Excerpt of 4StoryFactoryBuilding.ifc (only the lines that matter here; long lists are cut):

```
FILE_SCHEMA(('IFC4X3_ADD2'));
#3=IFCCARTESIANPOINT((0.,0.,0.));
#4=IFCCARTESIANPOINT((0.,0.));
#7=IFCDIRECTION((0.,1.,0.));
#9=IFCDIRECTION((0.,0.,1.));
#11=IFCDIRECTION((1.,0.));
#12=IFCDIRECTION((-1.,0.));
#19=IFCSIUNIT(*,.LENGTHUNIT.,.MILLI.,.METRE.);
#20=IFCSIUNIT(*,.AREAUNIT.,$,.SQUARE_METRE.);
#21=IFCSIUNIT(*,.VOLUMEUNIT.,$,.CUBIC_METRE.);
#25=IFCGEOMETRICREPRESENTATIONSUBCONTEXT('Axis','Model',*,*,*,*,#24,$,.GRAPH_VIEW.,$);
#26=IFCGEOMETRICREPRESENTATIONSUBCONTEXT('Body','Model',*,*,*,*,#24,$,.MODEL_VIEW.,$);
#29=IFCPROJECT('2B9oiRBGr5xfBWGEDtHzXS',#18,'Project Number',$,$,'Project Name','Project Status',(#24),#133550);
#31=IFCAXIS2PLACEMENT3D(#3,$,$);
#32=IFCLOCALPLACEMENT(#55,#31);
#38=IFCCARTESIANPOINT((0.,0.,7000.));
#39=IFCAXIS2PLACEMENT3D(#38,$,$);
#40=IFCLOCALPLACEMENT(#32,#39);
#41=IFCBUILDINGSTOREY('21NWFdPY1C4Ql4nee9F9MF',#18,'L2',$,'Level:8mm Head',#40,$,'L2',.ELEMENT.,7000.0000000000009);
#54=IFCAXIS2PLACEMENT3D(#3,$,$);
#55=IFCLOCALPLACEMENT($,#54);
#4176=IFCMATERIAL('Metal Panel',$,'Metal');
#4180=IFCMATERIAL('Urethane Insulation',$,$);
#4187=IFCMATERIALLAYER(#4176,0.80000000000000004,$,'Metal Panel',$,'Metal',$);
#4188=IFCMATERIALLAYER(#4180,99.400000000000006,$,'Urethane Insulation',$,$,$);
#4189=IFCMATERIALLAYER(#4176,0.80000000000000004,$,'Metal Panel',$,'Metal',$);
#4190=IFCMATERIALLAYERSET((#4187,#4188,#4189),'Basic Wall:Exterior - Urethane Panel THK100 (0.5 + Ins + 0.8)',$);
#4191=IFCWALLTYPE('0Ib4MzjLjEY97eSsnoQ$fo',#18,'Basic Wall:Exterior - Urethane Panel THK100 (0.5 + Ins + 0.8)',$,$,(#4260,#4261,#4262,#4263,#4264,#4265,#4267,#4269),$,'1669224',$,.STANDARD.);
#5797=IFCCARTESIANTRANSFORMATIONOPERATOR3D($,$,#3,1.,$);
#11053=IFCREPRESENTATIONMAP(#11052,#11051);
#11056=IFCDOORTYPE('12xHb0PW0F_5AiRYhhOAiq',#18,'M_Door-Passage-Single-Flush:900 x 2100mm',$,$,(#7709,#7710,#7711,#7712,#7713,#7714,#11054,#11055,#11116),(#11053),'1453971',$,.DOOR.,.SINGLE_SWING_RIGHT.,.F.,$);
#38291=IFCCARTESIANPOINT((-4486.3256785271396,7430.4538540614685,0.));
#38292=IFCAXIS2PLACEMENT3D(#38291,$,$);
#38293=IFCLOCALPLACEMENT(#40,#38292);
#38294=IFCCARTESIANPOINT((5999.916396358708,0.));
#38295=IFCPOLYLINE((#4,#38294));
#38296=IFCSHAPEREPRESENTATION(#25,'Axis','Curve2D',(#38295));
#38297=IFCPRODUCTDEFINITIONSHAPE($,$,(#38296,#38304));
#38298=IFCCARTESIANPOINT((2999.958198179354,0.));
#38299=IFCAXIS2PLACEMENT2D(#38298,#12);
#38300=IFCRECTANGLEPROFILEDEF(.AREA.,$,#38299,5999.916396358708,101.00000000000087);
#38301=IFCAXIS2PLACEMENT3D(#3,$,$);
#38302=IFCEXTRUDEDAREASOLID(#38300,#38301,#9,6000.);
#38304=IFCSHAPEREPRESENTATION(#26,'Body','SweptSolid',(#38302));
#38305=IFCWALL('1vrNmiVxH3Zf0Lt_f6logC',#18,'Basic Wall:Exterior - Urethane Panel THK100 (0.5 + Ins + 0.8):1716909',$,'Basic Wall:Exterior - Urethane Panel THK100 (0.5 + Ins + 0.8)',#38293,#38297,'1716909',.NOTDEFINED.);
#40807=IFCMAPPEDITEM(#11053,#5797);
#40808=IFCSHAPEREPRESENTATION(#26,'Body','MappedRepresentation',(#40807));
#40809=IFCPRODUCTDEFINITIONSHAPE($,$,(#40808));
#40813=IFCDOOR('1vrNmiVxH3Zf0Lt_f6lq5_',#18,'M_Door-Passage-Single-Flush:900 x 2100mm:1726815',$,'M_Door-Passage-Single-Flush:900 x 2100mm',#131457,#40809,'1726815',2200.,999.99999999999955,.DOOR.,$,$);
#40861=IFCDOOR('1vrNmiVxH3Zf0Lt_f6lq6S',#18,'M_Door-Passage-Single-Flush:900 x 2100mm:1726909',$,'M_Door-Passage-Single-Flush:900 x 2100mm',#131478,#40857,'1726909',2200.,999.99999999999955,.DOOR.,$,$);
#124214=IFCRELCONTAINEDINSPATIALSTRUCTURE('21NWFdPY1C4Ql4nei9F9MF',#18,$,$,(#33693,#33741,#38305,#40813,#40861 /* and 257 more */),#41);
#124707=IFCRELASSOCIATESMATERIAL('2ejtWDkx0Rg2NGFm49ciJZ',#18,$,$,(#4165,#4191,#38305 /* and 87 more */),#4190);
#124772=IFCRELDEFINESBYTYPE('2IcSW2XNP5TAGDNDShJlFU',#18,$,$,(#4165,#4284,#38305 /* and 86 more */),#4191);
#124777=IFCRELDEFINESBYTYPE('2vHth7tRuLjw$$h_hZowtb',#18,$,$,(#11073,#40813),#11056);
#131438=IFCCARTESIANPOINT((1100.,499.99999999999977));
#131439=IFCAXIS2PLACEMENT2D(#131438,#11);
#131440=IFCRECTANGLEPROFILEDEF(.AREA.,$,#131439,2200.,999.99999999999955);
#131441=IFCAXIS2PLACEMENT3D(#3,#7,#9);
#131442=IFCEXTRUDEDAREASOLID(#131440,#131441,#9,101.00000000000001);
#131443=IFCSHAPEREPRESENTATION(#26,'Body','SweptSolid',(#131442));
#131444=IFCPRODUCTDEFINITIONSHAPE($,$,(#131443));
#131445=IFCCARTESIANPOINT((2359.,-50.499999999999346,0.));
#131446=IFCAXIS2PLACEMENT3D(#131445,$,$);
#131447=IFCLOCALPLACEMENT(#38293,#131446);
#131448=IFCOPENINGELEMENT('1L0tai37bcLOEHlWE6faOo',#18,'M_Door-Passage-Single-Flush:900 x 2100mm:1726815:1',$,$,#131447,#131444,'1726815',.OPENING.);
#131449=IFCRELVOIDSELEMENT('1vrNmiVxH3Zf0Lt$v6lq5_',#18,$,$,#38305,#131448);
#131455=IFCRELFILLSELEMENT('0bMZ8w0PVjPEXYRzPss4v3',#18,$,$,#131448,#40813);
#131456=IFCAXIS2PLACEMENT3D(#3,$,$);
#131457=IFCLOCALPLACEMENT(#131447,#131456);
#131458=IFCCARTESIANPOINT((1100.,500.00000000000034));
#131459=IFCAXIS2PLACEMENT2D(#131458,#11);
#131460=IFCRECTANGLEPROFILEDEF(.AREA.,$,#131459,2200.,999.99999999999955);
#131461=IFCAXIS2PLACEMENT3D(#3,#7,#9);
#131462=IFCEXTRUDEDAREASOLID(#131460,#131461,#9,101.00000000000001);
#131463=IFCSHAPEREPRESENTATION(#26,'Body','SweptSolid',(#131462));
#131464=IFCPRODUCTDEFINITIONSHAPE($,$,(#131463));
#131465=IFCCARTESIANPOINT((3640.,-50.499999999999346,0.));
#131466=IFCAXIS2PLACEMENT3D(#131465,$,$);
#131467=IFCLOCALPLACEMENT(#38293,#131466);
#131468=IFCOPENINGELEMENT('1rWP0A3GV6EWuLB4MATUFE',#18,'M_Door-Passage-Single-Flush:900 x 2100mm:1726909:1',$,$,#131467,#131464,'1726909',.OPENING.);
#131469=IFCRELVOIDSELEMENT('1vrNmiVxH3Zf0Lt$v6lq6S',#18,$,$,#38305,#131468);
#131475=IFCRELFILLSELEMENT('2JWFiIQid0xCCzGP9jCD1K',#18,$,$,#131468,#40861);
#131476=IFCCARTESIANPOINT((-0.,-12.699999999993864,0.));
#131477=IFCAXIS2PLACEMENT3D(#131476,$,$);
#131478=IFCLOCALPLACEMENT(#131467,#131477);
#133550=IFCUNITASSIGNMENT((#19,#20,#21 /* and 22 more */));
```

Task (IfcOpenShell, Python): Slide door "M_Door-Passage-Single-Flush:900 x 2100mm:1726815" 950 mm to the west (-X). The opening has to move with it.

```python
import ifcopenshell
import ifcopenshell.api.geometry
import ifcopenshell.util.placement
import ifcopenshell.util.unit

model = ifcopenshell.open("4StoryFactoryBuilding.ifc")
unit_scale = ifcopenshell.util.unit.calculate_unit_scale(model)

door = model.by_guid("1vrNmiVxH3Zf0Lt_f6lq5_")
opening = door.FillsVoids[0].RelatingOpeningElement
wall = opening.VoidsElements[0].RelatingBuildingElement

wall_matrix = ifcopenshell.util.placement.get_local_placement(wall.ObjectPlacement)
shift = wall_matrix[:3, 0] * -0.95 / unit_scale
before = ifcopenshell.util.placement.get_local_placement(door.ObjectPlacement)[:3, 3].copy()

# The door is placed relative to its opening, so it follows when the opening moves.
matrix = ifcopenshell.util.placement.get_local_placement(opening.ObjectPlacement)
matrix[:3, 3] += shift
ifcopenshell.api.geometry.edit_object_placement(
    model, product=opening, matrix=matrix, is_si=False, should_transform_children=True
)

after = ifcopenshell.util.placement.get_local_placement(door.ObjectPlacement)[:3, 3]
print("door moved by", (after - before).round(3) + 0.0)

model.write("4StoryFactoryBuilding_rev.ifc")
```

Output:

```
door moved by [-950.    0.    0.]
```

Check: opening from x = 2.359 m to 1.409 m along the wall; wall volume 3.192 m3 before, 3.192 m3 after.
